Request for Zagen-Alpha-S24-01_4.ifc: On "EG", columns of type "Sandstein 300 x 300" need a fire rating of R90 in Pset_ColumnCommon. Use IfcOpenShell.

First a look at what the model holds.

```python
import ifcopenshell
import ifcopenshell.util.element

model = ifcopenshell.open("Zagen-Alpha-S24-01_4.ifc")
print(model.schema)
storey = next(s for s in model.by_type("IfcBuildingStorey") if s.Name == "EG")
columns = [e for e in ifcopenshell.util.element.get_decomposition(storey) if e.is_a("IfcColumn")]
seen = {}
for e in columns:
    element_type = ifcopenshell.util.element.get_type(e)
    key = (element_type.Name if element_type != e and element_type else None, ifcopenshell.util.element.get_pset(e, "Pset_ColumnCommon", "FireRating"))
    seen[key] = seen.get(key, 0) + 1
for (name, value), count in sorted(seen.items(), key=str):
    print(count, "x", name, "|", value)
```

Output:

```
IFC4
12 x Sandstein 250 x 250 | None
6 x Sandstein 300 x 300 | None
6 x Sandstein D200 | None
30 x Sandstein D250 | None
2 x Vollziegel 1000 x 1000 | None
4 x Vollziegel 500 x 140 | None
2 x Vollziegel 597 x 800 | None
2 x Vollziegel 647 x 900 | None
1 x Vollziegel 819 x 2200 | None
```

```python
import ifcopenshell
import ifcopenshell.api.pset
import ifcopenshell.util.element

model = ifcopenshell.open("Zagen-Alpha-S24-01_4.ifc")

storey = next(s for s in model.by_type("IfcBuildingStorey") if s.Name == "EG")
columns = [e for e in ifcopenshell.util.element.get_decomposition(storey) if e.is_a("IfcColumn")]

count = 0
for e in columns:
    element_type = ifcopenshell.util.element.get_type(e)
    if element_type in (None, e) or element_type.Name != "Sandstein 300 x 300":
        continue
    # add_pset returns the element's existing set when there is one.
    pset = ifcopenshell.api.pset.add_pset(model, product=e, name="Pset_ColumnCommon")
    ifcopenshell.api.pset.edit_pset(model, pset=pset, properties={"FireRating": "R90"})
    count += 1

print(count, "columns updated")

model.write("Zagen-Alpha-S24-01_4-out.ifc")
```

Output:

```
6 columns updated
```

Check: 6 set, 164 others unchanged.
